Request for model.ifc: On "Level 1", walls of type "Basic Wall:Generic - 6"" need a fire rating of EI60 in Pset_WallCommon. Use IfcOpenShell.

First a look at what the model holds.

```python
import ifcopenshell
import ifcopenshell.util.element

model = ifcopenshell.open("model.ifc")
print(model.schema)
storey = next(s for s in model.by_type("IfcBuildingStorey") if s.Name == "Level 1")
walls = [e for e in ifcopenshell.util.element.get_decomposition(storey) if e.is_a("IfcWall")]
seen = {}
for e in walls:
    element_type = ifcopenshell.util.element.get_type(e)
    key = (element_type.Name if element_type != e and element_type else None, ifcopenshell.util.element.get_pset(e, "Pset_WallCommon", "FireRating"))
    seen[key] = seen.get(key, 0) + 1
for (name, value), count in sorted(seen.items(), key=str):
    print(count, "x", name, "|", value)
```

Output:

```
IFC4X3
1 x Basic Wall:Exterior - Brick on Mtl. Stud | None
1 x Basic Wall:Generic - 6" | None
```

```python
import ifcopenshell
import ifcopenshell.api.pset
import ifcopenshell.util.element

model = ifcopenshell.open("model.ifc")

storey = next(s for s in model.by_type("IfcBuildingStorey") if s.Name == "Level 1")
walls = [e for e in ifcopenshell.util.element.get_decomposition(storey) if e.is_a("IfcWall")]

count = 0
for e in walls:
    element_type = ifcopenshell.util.element.get_type(e)
    if element_type in (None, e) or element_type.Name != 'Basic Wall:Generic - 6"':
        continue
    # add_pset returns the element's existing set when there is one.
    pset = ifcopenshell.api.pset.add_pset(model, product=e, name="Pset_WallCommon")
    ifcopenshell.api.pset.edit_pset(model, pset=pset, properties={"FireRating": "EI60"})
    count += 1

print(count, "walls updated")

model.write("model-out.ifc")
```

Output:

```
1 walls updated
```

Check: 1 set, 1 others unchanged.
